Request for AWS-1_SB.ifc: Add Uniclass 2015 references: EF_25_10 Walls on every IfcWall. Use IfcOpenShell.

First a look at what the model holds.

```python
import ifcopenshell

model = ifcopenshell.open("AWS-1_SB.ifc")
print(model.schema)
print("classifications:", [c.Name for c in model.by_type("IfcClassification")])
for ifc_class in ("IfcDoor", "IfcRoof", "IfcStair", "IfcWall", "IfcWindow"):
    print(ifc_class, len(model.by_type(ifc_class)))
```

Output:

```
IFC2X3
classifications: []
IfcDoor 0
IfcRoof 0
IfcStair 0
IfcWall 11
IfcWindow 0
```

```python
import ifcopenshell
import ifcopenshell.api.classification

model = ifcopenshell.open("AWS-1_SB.ifc")

# IFC2X3 requires Source and Edition and has no link from the project to the system.
system = model.create_entity("IfcClassification", Source="NBS", Edition="2015", Name="Uniclass 2015")

codes = {
    "IfcWall": ("EF_25_10", "Walls"),
}
for ifc_class, (code, name) in codes.items():
    products = model.by_type(ifc_class)
    ifcopenshell.api.classification.add_reference(
        model, products=products, classification=system, identification=code, name=name
    )
    print(code, len(products))

model.write("AWS-1_SB_updated.ifc")
```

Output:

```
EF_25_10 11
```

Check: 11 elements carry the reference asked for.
